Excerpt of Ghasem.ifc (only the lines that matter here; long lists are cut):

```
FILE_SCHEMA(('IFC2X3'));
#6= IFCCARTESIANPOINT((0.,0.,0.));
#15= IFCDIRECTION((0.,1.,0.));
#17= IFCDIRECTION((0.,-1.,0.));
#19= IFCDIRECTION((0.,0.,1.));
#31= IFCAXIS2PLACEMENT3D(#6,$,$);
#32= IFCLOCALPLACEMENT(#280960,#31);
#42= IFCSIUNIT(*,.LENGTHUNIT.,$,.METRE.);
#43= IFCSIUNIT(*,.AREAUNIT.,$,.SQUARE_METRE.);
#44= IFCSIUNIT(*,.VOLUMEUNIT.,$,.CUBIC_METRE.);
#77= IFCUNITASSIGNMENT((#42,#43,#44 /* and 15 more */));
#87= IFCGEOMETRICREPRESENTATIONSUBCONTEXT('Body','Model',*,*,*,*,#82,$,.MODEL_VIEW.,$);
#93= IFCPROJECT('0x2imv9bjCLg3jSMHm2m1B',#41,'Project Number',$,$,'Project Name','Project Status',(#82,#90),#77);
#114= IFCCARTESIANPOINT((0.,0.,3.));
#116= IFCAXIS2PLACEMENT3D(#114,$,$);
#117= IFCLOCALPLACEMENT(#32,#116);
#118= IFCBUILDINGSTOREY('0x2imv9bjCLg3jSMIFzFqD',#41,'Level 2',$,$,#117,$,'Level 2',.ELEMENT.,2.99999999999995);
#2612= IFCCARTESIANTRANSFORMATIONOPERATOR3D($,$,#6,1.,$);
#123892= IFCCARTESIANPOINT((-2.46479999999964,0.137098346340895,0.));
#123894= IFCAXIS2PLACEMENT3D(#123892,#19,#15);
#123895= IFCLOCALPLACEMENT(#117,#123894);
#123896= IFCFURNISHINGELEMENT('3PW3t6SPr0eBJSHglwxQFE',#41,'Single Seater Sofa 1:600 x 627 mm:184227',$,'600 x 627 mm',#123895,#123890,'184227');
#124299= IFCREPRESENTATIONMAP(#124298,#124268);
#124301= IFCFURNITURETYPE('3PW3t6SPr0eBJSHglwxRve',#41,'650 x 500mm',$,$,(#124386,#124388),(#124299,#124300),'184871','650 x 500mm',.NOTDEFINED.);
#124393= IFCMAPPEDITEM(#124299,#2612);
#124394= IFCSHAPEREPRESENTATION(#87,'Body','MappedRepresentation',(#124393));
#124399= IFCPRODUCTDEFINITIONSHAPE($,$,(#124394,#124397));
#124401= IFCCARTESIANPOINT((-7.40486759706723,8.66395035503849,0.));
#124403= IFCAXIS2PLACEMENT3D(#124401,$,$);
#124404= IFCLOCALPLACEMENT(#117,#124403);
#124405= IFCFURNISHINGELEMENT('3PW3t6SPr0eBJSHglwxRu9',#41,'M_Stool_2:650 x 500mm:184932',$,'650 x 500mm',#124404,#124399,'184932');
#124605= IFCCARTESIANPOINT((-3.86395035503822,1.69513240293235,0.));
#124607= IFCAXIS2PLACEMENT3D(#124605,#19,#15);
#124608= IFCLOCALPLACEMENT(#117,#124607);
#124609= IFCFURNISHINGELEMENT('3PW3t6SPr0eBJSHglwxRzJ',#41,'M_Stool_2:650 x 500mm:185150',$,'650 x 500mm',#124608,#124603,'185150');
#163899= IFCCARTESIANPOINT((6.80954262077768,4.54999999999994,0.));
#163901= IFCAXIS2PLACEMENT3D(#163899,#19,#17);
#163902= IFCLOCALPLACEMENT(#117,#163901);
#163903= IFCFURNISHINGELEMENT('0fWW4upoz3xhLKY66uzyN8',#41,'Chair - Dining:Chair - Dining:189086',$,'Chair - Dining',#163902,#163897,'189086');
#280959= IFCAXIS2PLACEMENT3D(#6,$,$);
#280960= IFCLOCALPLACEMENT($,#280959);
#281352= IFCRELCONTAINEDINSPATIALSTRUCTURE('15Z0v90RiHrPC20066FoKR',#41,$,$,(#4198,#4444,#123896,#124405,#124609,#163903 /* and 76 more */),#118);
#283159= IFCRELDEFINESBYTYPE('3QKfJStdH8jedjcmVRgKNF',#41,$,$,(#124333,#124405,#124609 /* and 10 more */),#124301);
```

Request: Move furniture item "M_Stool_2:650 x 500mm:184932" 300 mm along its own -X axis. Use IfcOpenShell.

```python
import ifcopenshell
import ifcopenshell.api.geometry
import ifcopenshell.util.placement
import ifcopenshell.util.unit

model = ifcopenshell.open("Ghasem.ifc")
unit_scale = ifcopenshell.util.unit.calculate_unit_scale(model)

item = model.by_guid("3PW3t6SPr0eBJSHglwxRu9")
matrix = ifcopenshell.util.placement.get_local_placement(item.ObjectPlacement)
matrix[:3, 3] -= matrix[:3, 0] * 0.3 / unit_scale
ifcopenshell.api.geometry.edit_object_placement(model, product=item, matrix=matrix, is_si=False)

print(ifcopenshell.util.placement.get_local_placement(item.ObjectPlacement).round(3) + 0.0)

model.write("Ghasem_edited.ifc")
```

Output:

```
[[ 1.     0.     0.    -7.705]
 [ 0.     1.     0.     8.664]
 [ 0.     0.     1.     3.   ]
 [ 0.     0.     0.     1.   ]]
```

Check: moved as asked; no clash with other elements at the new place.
